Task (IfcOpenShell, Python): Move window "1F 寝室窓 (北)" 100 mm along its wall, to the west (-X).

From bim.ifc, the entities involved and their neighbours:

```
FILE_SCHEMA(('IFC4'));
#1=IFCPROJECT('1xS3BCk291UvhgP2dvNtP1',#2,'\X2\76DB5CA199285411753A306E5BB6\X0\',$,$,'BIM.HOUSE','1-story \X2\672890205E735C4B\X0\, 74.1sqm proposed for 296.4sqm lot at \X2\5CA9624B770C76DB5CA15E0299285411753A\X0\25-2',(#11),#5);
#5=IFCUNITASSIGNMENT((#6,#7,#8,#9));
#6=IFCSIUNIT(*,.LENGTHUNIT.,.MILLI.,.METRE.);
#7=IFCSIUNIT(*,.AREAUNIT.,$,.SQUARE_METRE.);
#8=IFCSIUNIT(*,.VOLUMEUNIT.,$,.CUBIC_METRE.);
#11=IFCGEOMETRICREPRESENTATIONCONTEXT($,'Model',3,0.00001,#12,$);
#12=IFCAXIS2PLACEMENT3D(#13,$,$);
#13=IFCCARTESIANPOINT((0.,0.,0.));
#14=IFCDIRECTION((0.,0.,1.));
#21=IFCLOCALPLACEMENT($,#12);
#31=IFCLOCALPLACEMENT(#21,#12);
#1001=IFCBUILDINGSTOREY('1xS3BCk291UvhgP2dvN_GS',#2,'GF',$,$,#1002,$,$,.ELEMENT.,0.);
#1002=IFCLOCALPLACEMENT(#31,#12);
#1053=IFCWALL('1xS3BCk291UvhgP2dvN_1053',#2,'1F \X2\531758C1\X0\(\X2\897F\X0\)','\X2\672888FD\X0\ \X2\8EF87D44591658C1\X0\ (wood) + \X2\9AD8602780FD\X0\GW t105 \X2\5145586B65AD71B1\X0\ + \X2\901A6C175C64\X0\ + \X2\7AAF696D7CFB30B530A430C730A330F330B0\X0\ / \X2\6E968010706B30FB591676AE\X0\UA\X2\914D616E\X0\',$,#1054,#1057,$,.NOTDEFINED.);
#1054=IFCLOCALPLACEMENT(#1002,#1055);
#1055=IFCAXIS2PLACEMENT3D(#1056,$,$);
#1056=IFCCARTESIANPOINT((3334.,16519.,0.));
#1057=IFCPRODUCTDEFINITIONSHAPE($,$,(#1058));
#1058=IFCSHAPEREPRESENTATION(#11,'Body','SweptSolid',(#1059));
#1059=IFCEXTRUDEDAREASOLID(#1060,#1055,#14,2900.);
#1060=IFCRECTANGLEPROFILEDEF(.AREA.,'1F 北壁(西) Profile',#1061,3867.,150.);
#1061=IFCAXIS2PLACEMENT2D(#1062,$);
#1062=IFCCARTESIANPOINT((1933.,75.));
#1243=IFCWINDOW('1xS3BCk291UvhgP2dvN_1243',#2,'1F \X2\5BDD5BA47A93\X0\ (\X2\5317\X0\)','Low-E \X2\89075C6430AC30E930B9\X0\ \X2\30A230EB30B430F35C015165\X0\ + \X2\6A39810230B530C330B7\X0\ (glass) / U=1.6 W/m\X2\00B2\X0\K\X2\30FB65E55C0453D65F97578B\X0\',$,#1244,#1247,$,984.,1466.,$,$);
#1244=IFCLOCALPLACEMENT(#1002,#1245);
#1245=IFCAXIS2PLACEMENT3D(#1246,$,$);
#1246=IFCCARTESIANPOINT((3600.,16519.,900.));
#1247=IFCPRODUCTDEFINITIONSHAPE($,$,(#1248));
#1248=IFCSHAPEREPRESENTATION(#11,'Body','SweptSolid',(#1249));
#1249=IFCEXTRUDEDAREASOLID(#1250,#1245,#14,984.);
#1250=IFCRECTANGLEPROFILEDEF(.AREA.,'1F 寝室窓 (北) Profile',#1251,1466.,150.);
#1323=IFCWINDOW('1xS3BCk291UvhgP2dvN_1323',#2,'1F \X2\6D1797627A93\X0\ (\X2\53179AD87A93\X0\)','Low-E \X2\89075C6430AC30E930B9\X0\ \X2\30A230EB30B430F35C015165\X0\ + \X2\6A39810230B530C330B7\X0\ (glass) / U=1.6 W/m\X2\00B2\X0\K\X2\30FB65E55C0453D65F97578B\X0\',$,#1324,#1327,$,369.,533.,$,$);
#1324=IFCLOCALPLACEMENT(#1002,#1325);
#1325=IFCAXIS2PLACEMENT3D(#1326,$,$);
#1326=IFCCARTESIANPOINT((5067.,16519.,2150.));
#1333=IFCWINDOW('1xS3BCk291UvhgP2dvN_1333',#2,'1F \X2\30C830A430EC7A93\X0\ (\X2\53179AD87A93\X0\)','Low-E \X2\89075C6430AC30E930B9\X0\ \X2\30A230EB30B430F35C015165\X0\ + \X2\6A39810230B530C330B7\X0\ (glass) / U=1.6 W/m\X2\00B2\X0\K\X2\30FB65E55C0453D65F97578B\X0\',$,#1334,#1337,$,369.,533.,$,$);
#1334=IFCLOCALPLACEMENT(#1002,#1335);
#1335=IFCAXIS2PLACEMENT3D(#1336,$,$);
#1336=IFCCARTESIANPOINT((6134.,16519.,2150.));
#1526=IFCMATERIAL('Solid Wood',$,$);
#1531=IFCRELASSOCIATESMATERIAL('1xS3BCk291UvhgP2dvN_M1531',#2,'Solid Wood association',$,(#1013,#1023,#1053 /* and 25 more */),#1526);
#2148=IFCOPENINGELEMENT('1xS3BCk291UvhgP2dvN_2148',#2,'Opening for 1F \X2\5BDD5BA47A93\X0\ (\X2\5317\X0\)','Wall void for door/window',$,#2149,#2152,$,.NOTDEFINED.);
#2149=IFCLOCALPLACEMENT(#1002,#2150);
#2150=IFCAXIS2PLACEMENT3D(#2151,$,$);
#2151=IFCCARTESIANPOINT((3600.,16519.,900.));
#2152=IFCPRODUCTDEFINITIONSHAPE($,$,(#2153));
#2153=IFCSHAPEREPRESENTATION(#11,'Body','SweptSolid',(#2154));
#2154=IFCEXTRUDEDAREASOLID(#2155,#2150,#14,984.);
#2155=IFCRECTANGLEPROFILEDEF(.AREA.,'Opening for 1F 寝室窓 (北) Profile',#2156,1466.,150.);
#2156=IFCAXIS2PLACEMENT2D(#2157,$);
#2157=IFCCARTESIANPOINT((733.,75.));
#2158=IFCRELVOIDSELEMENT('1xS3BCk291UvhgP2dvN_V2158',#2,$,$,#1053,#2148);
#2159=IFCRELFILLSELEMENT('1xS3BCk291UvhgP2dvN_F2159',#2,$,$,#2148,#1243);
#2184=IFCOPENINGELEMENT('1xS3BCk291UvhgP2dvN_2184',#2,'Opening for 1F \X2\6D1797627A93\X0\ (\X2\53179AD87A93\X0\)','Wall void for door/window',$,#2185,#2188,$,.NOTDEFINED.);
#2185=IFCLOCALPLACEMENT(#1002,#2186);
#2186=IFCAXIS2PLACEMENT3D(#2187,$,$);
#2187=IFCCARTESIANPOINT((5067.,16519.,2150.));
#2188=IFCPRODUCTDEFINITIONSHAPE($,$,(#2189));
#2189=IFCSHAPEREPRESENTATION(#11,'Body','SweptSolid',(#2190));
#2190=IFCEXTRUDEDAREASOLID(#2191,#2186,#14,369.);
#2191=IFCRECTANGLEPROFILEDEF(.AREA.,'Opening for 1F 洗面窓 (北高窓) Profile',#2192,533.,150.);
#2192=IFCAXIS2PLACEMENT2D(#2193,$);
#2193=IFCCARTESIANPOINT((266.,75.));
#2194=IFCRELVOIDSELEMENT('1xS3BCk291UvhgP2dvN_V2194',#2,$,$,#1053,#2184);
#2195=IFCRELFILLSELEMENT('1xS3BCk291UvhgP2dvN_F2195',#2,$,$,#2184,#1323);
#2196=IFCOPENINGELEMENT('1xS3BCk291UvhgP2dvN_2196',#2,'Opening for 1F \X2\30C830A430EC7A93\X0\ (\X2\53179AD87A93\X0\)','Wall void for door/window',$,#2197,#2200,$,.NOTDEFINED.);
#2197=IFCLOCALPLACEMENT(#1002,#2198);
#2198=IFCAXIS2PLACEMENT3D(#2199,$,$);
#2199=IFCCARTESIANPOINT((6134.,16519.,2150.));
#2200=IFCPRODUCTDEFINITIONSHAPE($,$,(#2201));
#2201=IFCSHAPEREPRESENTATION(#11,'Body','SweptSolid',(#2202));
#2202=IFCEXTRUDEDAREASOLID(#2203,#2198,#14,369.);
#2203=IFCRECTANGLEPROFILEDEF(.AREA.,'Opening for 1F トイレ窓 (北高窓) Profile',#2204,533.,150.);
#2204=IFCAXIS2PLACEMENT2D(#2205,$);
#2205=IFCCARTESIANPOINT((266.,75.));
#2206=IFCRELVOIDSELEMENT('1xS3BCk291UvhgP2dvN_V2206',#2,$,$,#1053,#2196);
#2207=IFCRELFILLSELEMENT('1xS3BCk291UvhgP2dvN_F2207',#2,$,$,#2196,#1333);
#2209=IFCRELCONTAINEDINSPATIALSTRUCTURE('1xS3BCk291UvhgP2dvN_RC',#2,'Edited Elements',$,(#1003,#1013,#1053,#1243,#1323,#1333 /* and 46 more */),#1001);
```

```python
import ifcopenshell
import ifcopenshell.api.geometry
import ifcopenshell.util.placement
import ifcopenshell.util.unit

model = ifcopenshell.open("bim.ifc")
unit_scale = ifcopenshell.util.unit.calculate_unit_scale(model)

window = model.by_id(1243)
opening = window.FillsVoids[0].RelatingOpeningElement
wall = opening.VoidsElements[0].RelatingBuildingElement

wall_matrix = ifcopenshell.util.placement.get_local_placement(wall.ObjectPlacement)
shift = wall_matrix[:3, 0] * -0.1 / unit_scale
before = ifcopenshell.util.placement.get_local_placement(window.ObjectPlacement)[:3, 3].copy()

# The window is not placed relative to its opening, so move both.
for product in (opening, window):
    matrix = ifcopenshell.util.placement.get_local_placement(product.ObjectPlacement)
    matrix[:3, 3] += shift
    ifcopenshell.api.geometry.edit_object_placement(model, product=product, matrix=matrix, is_si=False)

after = ifcopenshell.util.placement.get_local_placement(window.ObjectPlacement)[:3, 3]
print("window moved by", (after - before).round(3) + 0.0)

model.write("bim_updated.ifc")
```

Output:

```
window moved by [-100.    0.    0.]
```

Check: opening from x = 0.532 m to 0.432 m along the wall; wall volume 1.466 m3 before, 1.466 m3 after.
